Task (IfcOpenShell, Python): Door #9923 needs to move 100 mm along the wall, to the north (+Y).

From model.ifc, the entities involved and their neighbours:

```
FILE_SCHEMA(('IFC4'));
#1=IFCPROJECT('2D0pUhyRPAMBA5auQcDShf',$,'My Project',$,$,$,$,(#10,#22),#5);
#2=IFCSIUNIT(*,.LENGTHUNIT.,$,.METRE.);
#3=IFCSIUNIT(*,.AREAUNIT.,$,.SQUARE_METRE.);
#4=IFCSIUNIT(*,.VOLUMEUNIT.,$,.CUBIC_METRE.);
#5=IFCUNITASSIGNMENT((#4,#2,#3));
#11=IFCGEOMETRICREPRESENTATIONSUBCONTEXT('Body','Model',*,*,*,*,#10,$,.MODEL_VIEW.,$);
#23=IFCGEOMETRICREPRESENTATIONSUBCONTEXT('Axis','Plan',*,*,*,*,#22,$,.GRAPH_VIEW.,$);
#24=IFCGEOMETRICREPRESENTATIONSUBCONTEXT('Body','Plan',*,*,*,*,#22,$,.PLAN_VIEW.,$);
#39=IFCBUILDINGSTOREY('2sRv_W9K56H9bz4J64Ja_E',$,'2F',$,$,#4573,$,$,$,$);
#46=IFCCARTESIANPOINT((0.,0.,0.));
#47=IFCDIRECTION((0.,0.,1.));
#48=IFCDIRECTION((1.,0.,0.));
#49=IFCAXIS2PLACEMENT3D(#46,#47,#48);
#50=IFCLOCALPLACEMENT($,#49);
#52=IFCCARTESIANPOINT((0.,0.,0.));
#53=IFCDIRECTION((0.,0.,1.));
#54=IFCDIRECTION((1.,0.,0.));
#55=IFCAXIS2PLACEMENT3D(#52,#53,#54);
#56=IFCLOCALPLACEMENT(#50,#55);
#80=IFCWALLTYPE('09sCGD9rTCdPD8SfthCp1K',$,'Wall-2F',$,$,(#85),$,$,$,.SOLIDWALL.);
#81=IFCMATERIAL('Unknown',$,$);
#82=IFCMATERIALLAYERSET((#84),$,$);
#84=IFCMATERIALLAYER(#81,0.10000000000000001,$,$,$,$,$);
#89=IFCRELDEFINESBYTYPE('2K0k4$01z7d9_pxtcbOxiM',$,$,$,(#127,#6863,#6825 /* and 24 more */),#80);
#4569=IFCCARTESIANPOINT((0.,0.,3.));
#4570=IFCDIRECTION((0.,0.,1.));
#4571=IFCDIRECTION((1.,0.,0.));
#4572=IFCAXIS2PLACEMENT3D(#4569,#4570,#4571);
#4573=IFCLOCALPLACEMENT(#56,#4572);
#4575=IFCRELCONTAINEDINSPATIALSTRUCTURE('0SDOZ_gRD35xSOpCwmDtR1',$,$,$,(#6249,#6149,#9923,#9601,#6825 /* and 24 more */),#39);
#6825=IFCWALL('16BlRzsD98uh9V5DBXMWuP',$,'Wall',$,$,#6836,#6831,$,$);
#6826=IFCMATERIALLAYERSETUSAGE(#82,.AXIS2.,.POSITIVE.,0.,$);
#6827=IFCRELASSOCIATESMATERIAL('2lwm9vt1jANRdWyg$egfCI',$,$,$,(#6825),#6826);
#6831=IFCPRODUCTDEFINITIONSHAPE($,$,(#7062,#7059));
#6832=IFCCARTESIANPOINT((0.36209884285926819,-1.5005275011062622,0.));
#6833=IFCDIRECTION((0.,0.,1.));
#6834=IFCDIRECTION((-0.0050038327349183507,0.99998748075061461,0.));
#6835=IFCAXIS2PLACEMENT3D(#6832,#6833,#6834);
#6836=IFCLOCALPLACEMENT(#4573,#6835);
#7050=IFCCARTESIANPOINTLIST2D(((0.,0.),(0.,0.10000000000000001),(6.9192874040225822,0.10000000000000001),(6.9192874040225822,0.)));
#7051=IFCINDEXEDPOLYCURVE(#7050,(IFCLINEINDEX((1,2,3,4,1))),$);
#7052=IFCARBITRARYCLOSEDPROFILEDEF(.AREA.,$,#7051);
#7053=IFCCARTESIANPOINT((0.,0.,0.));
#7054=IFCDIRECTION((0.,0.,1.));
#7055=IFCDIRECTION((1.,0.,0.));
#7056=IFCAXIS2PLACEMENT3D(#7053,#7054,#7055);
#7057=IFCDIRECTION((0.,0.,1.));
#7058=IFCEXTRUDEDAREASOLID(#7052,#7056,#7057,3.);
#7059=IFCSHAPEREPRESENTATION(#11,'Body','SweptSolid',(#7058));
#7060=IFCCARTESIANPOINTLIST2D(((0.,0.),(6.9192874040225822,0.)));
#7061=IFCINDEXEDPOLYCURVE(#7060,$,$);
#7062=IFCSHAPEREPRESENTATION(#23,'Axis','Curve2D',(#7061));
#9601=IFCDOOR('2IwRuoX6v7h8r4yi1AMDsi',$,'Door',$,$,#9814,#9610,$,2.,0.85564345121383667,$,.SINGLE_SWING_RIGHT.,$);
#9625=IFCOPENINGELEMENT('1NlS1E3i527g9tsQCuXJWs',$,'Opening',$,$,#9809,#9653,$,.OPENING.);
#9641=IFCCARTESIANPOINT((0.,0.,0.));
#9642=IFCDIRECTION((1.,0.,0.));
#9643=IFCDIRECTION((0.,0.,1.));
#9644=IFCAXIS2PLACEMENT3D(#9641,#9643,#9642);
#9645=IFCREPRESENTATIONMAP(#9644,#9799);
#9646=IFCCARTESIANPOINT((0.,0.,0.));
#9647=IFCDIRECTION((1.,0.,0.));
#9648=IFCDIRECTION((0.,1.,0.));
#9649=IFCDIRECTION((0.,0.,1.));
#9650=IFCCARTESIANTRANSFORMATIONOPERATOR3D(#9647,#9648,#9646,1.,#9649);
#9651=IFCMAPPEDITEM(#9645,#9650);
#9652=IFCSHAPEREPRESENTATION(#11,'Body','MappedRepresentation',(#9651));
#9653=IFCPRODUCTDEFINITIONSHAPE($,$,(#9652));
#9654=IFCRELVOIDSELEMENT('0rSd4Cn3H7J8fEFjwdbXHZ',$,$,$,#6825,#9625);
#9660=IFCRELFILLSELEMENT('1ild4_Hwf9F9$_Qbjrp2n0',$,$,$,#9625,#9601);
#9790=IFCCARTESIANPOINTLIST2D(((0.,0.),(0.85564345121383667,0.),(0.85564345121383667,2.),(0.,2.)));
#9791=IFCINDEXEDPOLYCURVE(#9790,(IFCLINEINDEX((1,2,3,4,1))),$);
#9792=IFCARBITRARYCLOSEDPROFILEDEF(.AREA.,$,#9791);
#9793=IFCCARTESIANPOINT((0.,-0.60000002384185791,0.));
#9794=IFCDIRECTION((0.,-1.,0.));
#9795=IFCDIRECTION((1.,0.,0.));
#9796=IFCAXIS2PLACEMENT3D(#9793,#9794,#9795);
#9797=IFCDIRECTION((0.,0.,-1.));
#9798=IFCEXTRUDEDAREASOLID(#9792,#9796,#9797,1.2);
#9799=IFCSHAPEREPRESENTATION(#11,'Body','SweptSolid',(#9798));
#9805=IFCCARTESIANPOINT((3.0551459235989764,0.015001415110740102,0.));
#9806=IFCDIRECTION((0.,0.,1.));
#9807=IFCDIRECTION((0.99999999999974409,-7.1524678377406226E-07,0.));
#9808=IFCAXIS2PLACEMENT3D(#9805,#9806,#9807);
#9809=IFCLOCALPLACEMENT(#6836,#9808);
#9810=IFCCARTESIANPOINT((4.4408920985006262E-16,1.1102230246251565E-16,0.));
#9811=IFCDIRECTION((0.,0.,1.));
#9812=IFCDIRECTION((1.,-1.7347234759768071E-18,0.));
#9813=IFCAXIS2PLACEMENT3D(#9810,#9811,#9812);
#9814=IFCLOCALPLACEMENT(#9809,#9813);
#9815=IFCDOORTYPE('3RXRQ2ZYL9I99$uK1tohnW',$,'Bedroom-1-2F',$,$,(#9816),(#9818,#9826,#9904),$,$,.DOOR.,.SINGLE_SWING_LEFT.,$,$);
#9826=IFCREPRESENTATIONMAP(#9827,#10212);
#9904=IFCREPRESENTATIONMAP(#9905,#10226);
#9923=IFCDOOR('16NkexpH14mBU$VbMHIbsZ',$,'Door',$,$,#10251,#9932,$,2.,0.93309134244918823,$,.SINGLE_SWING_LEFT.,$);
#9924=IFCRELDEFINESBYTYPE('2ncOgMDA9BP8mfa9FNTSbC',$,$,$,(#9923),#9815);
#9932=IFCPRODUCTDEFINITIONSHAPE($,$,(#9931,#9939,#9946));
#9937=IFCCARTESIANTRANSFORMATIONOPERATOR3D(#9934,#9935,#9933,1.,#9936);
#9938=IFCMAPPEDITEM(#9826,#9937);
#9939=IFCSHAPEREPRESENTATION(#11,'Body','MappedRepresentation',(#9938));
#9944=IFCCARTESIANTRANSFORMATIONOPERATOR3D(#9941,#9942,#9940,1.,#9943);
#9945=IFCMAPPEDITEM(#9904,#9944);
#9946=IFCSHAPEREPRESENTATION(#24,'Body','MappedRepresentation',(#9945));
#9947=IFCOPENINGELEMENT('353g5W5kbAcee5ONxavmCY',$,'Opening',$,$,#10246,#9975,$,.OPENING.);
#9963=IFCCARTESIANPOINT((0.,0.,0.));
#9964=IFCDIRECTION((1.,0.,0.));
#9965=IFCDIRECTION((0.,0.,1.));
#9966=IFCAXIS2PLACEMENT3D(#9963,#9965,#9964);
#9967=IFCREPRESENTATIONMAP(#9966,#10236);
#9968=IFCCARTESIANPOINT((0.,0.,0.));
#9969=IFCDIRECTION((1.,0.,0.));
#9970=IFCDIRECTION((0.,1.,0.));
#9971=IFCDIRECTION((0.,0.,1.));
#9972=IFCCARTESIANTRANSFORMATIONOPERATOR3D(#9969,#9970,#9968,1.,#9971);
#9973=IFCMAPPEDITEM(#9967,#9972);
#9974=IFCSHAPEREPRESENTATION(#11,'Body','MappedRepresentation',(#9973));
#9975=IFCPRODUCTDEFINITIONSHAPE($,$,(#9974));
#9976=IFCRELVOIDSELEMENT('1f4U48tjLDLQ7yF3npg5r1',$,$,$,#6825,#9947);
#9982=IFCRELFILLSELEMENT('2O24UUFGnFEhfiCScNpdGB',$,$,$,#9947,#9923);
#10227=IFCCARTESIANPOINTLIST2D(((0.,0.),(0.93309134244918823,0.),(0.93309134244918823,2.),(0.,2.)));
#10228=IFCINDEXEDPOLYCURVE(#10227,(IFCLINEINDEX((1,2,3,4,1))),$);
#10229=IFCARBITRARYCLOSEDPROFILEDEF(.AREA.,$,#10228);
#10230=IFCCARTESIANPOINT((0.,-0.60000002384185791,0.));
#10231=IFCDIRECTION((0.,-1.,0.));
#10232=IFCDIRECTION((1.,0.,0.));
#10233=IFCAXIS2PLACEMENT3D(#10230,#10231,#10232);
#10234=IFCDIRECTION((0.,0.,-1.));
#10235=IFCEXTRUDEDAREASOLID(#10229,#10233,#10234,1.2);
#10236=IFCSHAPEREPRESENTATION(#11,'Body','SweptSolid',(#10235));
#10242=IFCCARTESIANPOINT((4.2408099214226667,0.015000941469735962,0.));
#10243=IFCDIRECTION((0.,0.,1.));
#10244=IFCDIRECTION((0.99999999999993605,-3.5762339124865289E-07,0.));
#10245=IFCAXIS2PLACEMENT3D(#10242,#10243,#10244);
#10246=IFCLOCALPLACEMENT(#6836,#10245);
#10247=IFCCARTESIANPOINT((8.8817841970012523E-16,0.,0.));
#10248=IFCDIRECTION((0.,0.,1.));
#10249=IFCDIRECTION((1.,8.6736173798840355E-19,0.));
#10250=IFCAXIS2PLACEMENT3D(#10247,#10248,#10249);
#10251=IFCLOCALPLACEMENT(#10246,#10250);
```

```python
import ifcopenshell
import ifcopenshell.api.geometry
import ifcopenshell.util.placement
import ifcopenshell.util.unit

model = ifcopenshell.open("model.ifc")
unit_scale = ifcopenshell.util.unit.calculate_unit_scale(model)

door = model.by_guid("16NkexpH14mBU$VbMHIbsZ")
opening = door.FillsVoids[0].RelatingOpeningElement
wall = opening.VoidsElements[0].RelatingBuildingElement

wall_matrix = ifcopenshell.util.placement.get_local_placement(wall.ObjectPlacement)
shift = wall_matrix[:3, 0] * 0.1 / unit_scale
before = ifcopenshell.util.placement.get_local_placement(door.ObjectPlacement)[:3, 3].copy()

# The door is placed relative to its opening, so it follows when the opening moves.
matrix = ifcopenshell.util.placement.get_local_placement(opening.ObjectPlacement)
matrix[:3, 3] += shift
ifcopenshell.api.geometry.edit_object_placement(
    model, product=opening, matrix=matrix, is_si=False, should_transform_children=True
)

after = ifcopenshell.util.placement.get_local_placement(door.ObjectPlacement)[:3, 3]
print("door moved by", (after - before).round(3) + 0.0)

model.write("model_edited.ifc")
```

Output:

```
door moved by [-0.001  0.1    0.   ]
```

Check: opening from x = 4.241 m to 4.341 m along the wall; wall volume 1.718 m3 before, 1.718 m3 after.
